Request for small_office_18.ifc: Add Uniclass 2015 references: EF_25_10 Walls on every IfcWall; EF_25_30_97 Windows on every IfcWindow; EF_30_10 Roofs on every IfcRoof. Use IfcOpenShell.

First a look at what the model holds.

```python
import ifcopenshell

model = ifcopenshell.open("small_office_18.ifc")
print(model.schema)
print("classifications:", [c.Name for c in model.by_type("IfcClassification")])
for ifc_class in ("IfcDoor", "IfcRoof", "IfcStair", "IfcWall", "IfcWindow"):
    print(ifc_class, len(model.by_type(ifc_class)))
```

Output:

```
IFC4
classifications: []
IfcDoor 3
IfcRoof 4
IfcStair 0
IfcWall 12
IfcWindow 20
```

```python
import ifcopenshell
import ifcopenshell.api.classification

model = ifcopenshell.open("small_office_18.ifc")

system = ifcopenshell.api.classification.add_classification(model, classification="Uniclass 2015")

codes = {
    "IfcWall": ("EF_25_10", "Walls"),
    "IfcWindow": ("EF_25_30_97", "Windows"),
    "IfcRoof": ("EF_30_10", "Roofs"),
}
for ifc_class, (code, name) in codes.items():
    products = model.by_type(ifc_class)
    ifcopenshell.api.classification.add_reference(
        model, products=products, classification=system, identification=code, name=name
    )
    print(code, len(products))

model.write("small_office_18_rev.ifc")
```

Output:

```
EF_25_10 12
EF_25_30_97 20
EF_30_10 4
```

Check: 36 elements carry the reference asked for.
